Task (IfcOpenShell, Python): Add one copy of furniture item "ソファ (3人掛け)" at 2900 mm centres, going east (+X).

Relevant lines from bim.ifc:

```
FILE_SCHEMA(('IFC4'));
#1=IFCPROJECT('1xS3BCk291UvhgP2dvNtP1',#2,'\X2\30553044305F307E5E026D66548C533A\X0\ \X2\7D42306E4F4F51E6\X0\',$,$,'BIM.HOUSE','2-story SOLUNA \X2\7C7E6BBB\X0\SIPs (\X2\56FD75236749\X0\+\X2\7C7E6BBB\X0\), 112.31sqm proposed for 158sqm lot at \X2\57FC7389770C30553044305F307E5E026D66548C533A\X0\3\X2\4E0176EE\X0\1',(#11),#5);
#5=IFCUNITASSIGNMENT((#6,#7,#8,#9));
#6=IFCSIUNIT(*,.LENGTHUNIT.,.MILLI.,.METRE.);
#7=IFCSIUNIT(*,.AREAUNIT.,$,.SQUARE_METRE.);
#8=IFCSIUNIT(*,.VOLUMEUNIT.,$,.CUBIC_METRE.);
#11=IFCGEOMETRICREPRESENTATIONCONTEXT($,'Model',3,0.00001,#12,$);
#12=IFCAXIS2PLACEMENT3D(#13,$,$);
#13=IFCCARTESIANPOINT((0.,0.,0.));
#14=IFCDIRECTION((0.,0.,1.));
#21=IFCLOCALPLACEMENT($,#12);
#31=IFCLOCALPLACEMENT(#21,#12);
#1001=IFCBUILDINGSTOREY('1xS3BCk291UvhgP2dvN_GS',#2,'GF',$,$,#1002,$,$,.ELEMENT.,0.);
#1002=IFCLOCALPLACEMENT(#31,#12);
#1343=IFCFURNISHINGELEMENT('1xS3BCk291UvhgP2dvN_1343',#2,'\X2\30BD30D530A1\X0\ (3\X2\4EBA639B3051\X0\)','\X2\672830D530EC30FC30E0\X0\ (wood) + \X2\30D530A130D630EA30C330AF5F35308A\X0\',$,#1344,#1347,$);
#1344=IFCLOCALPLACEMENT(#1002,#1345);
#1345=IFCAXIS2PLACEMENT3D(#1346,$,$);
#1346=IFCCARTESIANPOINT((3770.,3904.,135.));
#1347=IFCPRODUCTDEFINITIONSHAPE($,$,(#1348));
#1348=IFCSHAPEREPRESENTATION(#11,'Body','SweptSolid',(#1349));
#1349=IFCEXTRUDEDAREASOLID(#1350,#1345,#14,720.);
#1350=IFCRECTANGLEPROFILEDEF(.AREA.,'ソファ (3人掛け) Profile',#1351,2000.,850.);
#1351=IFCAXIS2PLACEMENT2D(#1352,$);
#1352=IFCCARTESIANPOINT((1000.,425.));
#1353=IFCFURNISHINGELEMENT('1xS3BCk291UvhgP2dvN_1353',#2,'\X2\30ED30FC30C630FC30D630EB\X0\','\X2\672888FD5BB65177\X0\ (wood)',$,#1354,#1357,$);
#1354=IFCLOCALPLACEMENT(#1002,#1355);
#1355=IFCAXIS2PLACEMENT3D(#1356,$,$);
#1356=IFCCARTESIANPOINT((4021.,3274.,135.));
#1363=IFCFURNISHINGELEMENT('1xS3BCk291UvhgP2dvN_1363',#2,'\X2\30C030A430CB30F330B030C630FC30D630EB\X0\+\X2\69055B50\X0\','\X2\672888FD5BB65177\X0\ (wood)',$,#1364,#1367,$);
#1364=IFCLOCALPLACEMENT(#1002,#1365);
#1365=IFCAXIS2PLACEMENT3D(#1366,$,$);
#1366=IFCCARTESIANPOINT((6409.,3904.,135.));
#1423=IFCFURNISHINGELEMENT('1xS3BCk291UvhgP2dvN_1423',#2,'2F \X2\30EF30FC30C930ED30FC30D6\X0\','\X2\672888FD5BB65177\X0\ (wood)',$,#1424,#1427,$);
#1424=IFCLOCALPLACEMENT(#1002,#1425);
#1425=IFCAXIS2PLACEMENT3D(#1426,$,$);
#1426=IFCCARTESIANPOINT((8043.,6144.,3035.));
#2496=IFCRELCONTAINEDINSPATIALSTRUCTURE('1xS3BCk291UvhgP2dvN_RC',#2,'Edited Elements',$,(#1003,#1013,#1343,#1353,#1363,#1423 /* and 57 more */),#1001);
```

```python
import numpy as np
import ifcopenshell
import ifcopenshell.api.geometry
import ifcopenshell.api.root
import ifcopenshell.util.element
import ifcopenshell.util.placement

model = ifcopenshell.open("bim.ifc")


def reuse_history(source, copy):
    """copy_class also copies each property set's owner history, people and application; keep the originals."""
    for rel in copy.IsDefinedBy:
        if rel.is_a("IfcRelDefinesByProperties") and (history := rel.RelatingPropertyDefinition.OwnerHistory):
            rel.RelatingPropertyDefinition.OwnerHistory = source.OwnerHistory
            ifcopenshell.util.element.remove_deep2(model, history)


source = model.by_guid("1xS3BCk291UvhgP2dvN_1343")
base = ifcopenshell.util.placement.get_local_placement(source.ObjectPlacement)
step = np.array([1.0, 0.0, 0.0]) * 2900.0

for i in range(1, 2):
    copy = ifcopenshell.api.root.copy_class(model, product=source)
    copy.Representation = ifcopenshell.util.element.copy_deep(
        model, source.Representation, exclude=["IfcGeometricRepresentationContext", "IfcRepresentationMap"]
    )
    reuse_history(source, copy)
    matrix = base.copy()
    matrix[:3, 3] += i * step
    print("added at", matrix[:3, 3].round(3) + 0.0)
    ifcopenshell.api.geometry.edit_object_placement(model, product=copy, matrix=matrix, is_si=False)

model.write("bim_edited.ifc")
```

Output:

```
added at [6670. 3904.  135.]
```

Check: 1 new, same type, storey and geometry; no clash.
